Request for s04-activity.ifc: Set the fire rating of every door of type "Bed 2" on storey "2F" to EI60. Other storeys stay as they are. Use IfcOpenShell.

First a look at what the model holds.

```python
import ifcopenshell
import ifcopenshell.util.element

model = ifcopenshell.open("s04-activity.ifc")
print(model.schema)
storey = next(s for s in model.by_type("IfcBuildingStorey") if s.Name == "2F")
doors = [e for e in ifcopenshell.util.element.get_decomposition(storey) if e.is_a("IfcDoor")]
seen = {}
for e in doors:
    element_type = ifcopenshell.util.element.get_type(e)
    key = (element_type.Name if element_type != e and element_type else None, ifcopenshell.util.element.get_pset(e, "Pset_DoorCommon", "FireRating"))
    seen[key] = seen.get(key, 0) + 1
for (name, value), count in sorted(seen.items(), key=str):
    print(count, "x", name, "|", value)
```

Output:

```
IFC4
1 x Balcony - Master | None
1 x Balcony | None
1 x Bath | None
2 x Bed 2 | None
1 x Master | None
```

```python
import ifcopenshell
import ifcopenshell.api.pset
import ifcopenshell.util.element

model = ifcopenshell.open("s04-activity.ifc")

storey = next(s for s in model.by_type("IfcBuildingStorey") if s.Name == "2F")
doors = [e for e in ifcopenshell.util.element.get_decomposition(storey) if e.is_a("IfcDoor")]

count = 0
for e in doors:
    element_type = ifcopenshell.util.element.get_type(e)
    if element_type in (None, e) or element_type.Name != "Bed 2":
        continue
    # add_pset returns the element's existing set when there is one.
    pset = ifcopenshell.api.pset.add_pset(model, product=e, name="Pset_DoorCommon")
    ifcopenshell.api.pset.edit_pset(model, pset=pset, properties={"FireRating": "EI60"})
    count += 1

print(count, "doors updated")

model.write("s04-activity-out.ifc")
```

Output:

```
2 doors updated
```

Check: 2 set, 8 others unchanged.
